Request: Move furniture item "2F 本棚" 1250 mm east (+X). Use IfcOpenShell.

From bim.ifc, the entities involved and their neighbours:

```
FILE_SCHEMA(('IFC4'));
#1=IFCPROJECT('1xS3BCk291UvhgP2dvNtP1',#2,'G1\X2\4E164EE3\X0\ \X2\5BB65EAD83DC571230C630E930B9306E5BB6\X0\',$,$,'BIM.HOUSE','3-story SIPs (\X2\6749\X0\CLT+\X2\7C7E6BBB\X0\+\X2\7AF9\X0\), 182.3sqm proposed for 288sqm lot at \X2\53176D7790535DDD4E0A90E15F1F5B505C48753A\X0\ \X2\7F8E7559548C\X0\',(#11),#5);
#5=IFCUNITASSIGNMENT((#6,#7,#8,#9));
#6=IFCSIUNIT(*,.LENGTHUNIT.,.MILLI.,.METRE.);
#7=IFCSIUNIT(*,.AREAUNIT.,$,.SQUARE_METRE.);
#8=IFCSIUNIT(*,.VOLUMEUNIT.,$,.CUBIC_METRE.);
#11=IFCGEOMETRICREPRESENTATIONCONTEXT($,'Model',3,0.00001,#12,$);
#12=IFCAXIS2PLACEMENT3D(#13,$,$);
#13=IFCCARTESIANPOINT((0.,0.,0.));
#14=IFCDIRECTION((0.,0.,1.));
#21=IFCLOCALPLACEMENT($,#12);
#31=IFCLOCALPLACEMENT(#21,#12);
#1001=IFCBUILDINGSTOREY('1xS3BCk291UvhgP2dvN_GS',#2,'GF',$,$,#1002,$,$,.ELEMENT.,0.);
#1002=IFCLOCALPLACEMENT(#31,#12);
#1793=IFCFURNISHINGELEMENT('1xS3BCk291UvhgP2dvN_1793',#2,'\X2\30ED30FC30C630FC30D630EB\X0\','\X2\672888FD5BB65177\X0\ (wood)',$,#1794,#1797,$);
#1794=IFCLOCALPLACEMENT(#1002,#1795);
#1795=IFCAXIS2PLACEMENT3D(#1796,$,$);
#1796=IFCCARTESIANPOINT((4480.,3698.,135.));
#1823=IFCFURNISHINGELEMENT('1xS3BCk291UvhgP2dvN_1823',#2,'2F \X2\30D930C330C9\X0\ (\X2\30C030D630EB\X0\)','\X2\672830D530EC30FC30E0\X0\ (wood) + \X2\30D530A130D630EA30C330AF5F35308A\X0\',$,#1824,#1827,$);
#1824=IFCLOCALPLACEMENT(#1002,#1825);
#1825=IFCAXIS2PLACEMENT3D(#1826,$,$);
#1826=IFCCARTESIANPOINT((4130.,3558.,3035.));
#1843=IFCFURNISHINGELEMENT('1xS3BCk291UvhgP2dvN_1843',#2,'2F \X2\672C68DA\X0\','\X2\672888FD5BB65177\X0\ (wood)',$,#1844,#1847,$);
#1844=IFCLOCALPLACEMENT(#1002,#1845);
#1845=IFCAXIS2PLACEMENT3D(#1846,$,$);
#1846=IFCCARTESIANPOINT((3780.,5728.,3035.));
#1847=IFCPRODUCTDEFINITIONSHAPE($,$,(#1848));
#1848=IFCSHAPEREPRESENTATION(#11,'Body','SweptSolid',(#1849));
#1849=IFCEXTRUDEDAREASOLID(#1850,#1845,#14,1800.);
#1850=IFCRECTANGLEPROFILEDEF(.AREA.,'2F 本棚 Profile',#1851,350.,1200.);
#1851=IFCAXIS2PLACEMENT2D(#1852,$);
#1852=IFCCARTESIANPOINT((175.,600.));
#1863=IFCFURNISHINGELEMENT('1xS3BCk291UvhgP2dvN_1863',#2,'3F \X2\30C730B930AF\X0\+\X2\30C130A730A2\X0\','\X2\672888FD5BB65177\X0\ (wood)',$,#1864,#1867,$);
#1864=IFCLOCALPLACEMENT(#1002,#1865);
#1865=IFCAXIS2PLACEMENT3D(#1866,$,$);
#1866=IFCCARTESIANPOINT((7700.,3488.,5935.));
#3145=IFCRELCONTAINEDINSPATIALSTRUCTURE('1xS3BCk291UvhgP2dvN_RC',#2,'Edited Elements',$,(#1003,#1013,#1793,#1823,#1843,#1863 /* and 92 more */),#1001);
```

```python
import ifcopenshell
import ifcopenshell.api.geometry
import ifcopenshell.util.placement
import ifcopenshell.util.unit

model = ifcopenshell.open("bim.ifc")
unit_scale = ifcopenshell.util.unit.calculate_unit_scale(model)

item = model.by_guid("1xS3BCk291UvhgP2dvN_1843")
matrix = ifcopenshell.util.placement.get_local_placement(item.ObjectPlacement)
matrix[0, 3] += 1.25 / unit_scale
ifcopenshell.api.geometry.edit_object_placement(model, product=item, matrix=matrix, is_si=False)

print(ifcopenshell.util.placement.get_local_placement(item.ObjectPlacement).round(3) + 0.0)

model.write("bim_edited.ifc")
```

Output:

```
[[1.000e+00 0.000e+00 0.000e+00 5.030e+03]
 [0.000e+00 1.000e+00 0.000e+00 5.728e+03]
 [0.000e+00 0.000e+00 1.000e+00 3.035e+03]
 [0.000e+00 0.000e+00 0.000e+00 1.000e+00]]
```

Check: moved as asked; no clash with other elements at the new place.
